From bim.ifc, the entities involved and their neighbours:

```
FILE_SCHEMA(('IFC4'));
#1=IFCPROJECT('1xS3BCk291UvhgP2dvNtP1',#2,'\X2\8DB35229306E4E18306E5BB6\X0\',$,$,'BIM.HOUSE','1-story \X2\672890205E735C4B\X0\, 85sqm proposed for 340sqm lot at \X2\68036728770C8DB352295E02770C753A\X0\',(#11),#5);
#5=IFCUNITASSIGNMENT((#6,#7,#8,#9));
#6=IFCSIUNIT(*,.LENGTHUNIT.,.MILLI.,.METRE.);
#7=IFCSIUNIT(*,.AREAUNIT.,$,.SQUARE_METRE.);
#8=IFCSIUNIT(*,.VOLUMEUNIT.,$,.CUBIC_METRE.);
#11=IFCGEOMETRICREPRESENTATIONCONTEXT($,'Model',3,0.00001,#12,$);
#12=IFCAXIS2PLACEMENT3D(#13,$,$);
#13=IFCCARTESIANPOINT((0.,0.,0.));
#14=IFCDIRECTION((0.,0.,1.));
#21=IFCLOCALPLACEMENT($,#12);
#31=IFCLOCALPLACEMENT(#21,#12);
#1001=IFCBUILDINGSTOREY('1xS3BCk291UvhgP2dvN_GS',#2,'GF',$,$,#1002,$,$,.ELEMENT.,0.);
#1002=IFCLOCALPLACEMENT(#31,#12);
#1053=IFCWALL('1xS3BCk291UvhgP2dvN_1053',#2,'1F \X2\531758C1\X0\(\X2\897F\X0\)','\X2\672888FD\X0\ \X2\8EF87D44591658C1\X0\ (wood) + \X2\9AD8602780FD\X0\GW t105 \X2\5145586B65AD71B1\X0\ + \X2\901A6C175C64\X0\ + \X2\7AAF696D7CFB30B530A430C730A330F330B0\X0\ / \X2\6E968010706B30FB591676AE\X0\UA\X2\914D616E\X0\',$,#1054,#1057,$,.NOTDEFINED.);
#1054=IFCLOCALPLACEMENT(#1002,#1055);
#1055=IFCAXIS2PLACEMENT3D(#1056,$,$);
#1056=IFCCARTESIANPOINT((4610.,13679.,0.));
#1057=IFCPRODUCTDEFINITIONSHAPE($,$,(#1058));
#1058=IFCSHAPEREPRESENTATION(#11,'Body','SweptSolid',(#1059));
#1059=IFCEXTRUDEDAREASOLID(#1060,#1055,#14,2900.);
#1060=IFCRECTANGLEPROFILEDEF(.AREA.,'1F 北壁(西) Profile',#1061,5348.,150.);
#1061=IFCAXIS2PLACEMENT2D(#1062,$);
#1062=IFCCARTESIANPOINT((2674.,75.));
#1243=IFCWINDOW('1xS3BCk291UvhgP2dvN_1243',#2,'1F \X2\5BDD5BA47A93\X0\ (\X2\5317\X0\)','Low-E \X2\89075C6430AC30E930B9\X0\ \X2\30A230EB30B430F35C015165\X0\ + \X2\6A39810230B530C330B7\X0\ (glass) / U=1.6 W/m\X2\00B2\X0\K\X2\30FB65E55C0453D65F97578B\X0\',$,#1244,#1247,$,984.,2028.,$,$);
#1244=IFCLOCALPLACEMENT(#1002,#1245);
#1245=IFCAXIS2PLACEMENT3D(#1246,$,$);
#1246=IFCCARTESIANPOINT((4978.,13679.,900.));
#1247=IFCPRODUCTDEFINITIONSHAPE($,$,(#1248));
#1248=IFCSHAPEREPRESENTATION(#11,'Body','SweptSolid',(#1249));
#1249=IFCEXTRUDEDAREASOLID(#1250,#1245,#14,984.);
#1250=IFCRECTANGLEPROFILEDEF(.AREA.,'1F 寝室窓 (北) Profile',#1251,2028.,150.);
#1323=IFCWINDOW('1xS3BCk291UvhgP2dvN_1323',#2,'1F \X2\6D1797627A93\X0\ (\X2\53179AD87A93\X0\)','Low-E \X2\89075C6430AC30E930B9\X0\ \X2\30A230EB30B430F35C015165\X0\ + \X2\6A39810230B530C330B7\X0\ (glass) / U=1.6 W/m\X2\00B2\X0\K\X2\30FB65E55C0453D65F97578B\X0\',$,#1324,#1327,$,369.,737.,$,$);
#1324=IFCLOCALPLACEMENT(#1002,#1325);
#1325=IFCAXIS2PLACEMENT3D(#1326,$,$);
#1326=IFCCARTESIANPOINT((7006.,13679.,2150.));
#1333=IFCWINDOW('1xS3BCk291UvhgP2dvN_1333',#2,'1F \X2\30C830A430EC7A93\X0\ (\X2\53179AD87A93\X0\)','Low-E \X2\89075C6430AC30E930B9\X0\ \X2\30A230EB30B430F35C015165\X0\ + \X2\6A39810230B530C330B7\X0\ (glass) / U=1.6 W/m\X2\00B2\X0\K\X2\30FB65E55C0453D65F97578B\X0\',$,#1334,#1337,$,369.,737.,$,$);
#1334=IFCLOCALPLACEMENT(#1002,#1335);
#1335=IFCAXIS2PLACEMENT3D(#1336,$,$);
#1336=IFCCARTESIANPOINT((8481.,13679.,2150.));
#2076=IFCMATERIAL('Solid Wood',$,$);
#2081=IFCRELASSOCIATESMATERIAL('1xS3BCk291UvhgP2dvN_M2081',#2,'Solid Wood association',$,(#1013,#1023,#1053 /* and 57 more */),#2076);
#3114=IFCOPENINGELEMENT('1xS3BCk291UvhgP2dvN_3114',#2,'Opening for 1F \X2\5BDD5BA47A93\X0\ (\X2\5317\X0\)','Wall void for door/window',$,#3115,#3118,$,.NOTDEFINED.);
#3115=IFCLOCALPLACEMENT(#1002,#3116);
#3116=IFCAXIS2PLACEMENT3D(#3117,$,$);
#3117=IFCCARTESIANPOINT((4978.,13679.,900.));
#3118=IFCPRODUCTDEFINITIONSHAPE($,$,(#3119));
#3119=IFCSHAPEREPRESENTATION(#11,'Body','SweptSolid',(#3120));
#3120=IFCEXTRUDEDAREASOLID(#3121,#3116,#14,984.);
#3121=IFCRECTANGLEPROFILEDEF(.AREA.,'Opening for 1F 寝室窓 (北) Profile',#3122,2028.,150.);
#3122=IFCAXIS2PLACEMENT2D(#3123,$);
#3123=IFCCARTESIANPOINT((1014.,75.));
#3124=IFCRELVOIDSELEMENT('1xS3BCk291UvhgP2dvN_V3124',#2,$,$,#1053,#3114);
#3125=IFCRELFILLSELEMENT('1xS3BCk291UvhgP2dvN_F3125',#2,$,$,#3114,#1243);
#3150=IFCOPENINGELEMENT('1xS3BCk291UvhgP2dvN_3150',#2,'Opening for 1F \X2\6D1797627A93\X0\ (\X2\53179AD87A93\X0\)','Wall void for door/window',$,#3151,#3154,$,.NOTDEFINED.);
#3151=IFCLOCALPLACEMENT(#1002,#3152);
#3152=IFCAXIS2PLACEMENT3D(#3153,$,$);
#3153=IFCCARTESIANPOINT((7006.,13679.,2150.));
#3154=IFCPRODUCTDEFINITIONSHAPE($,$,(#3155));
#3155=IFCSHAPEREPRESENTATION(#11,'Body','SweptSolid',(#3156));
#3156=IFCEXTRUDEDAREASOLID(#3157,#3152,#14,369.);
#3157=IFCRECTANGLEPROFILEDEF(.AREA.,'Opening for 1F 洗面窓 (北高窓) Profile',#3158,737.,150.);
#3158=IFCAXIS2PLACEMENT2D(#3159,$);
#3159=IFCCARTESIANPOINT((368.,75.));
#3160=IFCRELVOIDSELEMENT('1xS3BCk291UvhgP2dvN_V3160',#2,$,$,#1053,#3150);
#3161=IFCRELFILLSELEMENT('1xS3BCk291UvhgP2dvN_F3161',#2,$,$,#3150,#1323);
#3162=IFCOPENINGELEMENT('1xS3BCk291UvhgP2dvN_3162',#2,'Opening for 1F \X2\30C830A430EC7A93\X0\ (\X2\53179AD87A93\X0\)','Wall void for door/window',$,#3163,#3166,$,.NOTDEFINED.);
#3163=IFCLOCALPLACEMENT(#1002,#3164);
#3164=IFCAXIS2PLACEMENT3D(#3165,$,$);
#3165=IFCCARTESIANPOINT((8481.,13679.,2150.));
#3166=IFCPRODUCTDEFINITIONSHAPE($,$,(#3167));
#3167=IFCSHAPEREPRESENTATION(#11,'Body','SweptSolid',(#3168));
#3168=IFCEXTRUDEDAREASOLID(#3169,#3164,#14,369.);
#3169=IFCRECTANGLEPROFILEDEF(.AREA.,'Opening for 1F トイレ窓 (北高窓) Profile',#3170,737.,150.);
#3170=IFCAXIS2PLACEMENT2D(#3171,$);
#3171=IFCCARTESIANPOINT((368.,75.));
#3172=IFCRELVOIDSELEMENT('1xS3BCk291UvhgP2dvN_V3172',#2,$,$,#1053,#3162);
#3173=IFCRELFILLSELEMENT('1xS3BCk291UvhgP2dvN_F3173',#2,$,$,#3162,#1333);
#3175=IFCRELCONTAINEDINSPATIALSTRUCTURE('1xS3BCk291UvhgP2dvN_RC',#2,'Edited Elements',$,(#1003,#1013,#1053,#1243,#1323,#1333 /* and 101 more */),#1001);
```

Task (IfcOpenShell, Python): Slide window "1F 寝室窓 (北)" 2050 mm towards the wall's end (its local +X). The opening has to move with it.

```python
import ifcopenshell
import ifcopenshell.api.geometry
import ifcopenshell.util.placement
import ifcopenshell.util.unit

model = ifcopenshell.open("bim.ifc")
unit_scale = ifcopenshell.util.unit.calculate_unit_scale(model)

window = model.by_guid("1xS3BCk291UvhgP2dvN_1243")
opening = window.FillsVoids[0].RelatingOpeningElement
wall = opening.VoidsElements[0].RelatingBuildingElement

wall_matrix = ifcopenshell.util.placement.get_local_placement(wall.ObjectPlacement)
shift = wall_matrix[:3, 0] * 2.05 / unit_scale
before = ifcopenshell.util.placement.get_local_placement(window.ObjectPlacement)[:3, 3].copy()

# The window is not placed relative to its opening, so move both.
for product in (opening, window):
    matrix = ifcopenshell.util.placement.get_local_placement(product.ObjectPlacement)
    matrix[:3, 3] += shift
    ifcopenshell.api.geometry.edit_object_placement(model, product=product, matrix=matrix, is_si=False)

after = ifcopenshell.util.placement.get_local_placement(window.ObjectPlacement)[:3, 3]
print("window moved by", (after - before).round(3) + 0.0)

model.write("bim_edited.ifc")
```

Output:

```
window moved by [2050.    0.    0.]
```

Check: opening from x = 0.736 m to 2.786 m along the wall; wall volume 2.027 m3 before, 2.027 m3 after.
